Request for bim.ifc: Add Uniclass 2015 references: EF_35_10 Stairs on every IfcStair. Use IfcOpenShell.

First a look at what the model holds.

```python
import ifcopenshell

model = ifcopenshell.open("bim.ifc")
print(model.schema)
print("classifications:", [c.Name for c in model.by_type("IfcClassification")])
for ifc_class in ("IfcDoor", "IfcRoof", "IfcStair", "IfcWall", "IfcWindow"):
    print(ifc_class, len(model.by_type(ifc_class)))
```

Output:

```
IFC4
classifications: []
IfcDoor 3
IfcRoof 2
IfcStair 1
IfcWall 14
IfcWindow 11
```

```python
import ifcopenshell
import ifcopenshell.api.classification

model = ifcopenshell.open("bim.ifc")

system = ifcopenshell.api.classification.add_classification(model, classification="Uniclass 2015")

codes = {
    "IfcStair": ("EF_35_10", "Stairs"),
}
for ifc_class, (code, name) in codes.items():
    products = model.by_type(ifc_class)
    ifcopenshell.api.classification.add_reference(
        model, products=products, classification=system, identification=code, name=name
    )
    print(code, len(products))

model.write("bim_rev.ifc")
```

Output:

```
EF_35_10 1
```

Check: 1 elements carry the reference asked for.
